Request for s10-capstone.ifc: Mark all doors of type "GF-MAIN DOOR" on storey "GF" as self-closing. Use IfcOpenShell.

First a look at what the model holds.

```python
import ifcopenshell
import ifcopenshell.util.element

model = ifcopenshell.open("s10-capstone.ifc")
print(model.schema)
storey = next(s for s in model.by_type("IfcBuildingStorey") if s.Name == "GF")
doors = [e for e in ifcopenshell.util.element.get_decomposition(storey) if e.is_a("IfcDoor")]
seen = {}
for e in doors:
    element_type = ifcopenshell.util.element.get_type(e)
    key = (element_type.Name if element_type != e and element_type else None, ifcopenshell.util.element.get_pset(e, "Pset_DoorCommon", "SelfClosing"))
    seen[key] = seen.get(key, 0) + 1
for (name, value), count in sorted(seen.items(), key=str):
    print(count, "x", name, "|", value)
```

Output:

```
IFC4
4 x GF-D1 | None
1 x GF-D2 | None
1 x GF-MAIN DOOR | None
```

```python
import ifcopenshell
import ifcopenshell.api.pset
import ifcopenshell.util.element

model = ifcopenshell.open("s10-capstone.ifc")

storey = next(s for s in model.by_type("IfcBuildingStorey") if s.Name == "GF")
doors = [e for e in ifcopenshell.util.element.get_decomposition(storey) if e.is_a("IfcDoor")]

count = 0
for e in doors:
    element_type = ifcopenshell.util.element.get_type(e)
    if element_type in (None, e) or element_type.Name != "GF-MAIN DOOR":
        continue
    # add_pset returns the element's existing set when there is one.
    pset = ifcopenshell.api.pset.add_pset(model, product=e, name="Pset_DoorCommon")
    ifcopenshell.api.pset.edit_pset(model, pset=pset, properties={"SelfClosing": True})
    count += 1

print(count, "doors updated")

model.write("s10-capstone_updated.ifc")
```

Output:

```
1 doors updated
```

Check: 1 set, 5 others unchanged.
